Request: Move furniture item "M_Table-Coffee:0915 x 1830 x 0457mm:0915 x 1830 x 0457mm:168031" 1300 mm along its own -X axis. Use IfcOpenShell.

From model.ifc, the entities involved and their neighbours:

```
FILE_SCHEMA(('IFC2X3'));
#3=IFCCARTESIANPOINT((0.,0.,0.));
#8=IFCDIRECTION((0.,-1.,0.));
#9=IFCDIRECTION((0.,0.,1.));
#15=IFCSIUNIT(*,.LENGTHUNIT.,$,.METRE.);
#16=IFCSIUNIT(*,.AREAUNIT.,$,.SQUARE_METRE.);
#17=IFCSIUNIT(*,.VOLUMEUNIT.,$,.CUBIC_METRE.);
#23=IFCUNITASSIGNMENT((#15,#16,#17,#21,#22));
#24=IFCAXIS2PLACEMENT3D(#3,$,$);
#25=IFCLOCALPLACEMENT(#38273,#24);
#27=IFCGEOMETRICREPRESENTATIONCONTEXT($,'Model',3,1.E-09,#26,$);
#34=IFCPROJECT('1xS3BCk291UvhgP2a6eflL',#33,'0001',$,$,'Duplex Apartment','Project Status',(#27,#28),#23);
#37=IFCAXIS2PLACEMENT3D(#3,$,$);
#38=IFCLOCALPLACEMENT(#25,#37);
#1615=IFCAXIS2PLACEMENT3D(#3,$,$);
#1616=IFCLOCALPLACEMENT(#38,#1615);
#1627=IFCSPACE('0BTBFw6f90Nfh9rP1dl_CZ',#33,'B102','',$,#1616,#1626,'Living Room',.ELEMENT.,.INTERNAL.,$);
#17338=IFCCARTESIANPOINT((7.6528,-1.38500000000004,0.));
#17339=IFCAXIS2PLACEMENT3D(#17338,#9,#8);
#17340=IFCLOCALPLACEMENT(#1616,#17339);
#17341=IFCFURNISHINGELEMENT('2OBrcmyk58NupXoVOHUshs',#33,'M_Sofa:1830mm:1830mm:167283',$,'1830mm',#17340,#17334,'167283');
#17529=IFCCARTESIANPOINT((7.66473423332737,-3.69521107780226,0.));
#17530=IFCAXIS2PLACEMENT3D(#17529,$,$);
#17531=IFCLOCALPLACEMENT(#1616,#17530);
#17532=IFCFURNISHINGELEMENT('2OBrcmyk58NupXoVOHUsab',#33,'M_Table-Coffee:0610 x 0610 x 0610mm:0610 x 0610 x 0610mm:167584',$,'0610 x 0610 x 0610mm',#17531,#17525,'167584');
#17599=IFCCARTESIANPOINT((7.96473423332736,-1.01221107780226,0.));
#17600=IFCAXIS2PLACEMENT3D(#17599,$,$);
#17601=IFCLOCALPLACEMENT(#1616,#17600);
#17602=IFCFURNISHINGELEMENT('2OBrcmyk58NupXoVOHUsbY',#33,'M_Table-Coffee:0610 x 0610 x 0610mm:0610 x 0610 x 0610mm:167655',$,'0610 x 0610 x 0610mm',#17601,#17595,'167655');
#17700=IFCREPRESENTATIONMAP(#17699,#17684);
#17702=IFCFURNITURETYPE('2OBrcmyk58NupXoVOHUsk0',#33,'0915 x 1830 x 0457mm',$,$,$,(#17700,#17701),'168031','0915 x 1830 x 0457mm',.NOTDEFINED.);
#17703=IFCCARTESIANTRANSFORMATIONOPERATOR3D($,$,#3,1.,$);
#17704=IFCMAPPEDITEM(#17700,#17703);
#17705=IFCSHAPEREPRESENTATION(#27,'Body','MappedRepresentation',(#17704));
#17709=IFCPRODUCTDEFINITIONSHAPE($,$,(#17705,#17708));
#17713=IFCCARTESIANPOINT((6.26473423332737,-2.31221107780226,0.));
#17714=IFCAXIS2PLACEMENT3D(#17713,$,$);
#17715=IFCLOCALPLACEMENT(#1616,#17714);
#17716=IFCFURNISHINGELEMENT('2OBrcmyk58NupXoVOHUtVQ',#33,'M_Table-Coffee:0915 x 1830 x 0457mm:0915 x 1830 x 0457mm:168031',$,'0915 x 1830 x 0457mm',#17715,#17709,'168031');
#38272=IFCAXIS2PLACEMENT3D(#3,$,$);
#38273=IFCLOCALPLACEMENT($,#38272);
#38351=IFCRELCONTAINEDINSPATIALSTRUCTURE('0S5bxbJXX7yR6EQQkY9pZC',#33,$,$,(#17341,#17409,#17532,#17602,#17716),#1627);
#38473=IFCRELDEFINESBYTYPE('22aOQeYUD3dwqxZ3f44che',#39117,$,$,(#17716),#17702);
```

```python
import ifcopenshell
import ifcopenshell.api.geometry
import ifcopenshell.util.placement
import ifcopenshell.util.unit

model = ifcopenshell.open("model.ifc")
unit_scale = ifcopenshell.util.unit.calculate_unit_scale(model)

item = model.by_id(17716)
matrix = ifcopenshell.util.placement.get_local_placement(item.ObjectPlacement)
matrix[:3, 3] -= matrix[:3, 0] * 1.3 / unit_scale
ifcopenshell.api.geometry.edit_object_placement(model, product=item, matrix=matrix, is_si=False)

print(ifcopenshell.util.placement.get_local_placement(item.ObjectPlacement).round(3) + 0.0)

model.write("model_edited.ifc")
```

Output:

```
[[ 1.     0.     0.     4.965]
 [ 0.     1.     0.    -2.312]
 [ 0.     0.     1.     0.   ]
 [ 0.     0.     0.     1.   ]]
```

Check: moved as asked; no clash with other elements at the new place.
